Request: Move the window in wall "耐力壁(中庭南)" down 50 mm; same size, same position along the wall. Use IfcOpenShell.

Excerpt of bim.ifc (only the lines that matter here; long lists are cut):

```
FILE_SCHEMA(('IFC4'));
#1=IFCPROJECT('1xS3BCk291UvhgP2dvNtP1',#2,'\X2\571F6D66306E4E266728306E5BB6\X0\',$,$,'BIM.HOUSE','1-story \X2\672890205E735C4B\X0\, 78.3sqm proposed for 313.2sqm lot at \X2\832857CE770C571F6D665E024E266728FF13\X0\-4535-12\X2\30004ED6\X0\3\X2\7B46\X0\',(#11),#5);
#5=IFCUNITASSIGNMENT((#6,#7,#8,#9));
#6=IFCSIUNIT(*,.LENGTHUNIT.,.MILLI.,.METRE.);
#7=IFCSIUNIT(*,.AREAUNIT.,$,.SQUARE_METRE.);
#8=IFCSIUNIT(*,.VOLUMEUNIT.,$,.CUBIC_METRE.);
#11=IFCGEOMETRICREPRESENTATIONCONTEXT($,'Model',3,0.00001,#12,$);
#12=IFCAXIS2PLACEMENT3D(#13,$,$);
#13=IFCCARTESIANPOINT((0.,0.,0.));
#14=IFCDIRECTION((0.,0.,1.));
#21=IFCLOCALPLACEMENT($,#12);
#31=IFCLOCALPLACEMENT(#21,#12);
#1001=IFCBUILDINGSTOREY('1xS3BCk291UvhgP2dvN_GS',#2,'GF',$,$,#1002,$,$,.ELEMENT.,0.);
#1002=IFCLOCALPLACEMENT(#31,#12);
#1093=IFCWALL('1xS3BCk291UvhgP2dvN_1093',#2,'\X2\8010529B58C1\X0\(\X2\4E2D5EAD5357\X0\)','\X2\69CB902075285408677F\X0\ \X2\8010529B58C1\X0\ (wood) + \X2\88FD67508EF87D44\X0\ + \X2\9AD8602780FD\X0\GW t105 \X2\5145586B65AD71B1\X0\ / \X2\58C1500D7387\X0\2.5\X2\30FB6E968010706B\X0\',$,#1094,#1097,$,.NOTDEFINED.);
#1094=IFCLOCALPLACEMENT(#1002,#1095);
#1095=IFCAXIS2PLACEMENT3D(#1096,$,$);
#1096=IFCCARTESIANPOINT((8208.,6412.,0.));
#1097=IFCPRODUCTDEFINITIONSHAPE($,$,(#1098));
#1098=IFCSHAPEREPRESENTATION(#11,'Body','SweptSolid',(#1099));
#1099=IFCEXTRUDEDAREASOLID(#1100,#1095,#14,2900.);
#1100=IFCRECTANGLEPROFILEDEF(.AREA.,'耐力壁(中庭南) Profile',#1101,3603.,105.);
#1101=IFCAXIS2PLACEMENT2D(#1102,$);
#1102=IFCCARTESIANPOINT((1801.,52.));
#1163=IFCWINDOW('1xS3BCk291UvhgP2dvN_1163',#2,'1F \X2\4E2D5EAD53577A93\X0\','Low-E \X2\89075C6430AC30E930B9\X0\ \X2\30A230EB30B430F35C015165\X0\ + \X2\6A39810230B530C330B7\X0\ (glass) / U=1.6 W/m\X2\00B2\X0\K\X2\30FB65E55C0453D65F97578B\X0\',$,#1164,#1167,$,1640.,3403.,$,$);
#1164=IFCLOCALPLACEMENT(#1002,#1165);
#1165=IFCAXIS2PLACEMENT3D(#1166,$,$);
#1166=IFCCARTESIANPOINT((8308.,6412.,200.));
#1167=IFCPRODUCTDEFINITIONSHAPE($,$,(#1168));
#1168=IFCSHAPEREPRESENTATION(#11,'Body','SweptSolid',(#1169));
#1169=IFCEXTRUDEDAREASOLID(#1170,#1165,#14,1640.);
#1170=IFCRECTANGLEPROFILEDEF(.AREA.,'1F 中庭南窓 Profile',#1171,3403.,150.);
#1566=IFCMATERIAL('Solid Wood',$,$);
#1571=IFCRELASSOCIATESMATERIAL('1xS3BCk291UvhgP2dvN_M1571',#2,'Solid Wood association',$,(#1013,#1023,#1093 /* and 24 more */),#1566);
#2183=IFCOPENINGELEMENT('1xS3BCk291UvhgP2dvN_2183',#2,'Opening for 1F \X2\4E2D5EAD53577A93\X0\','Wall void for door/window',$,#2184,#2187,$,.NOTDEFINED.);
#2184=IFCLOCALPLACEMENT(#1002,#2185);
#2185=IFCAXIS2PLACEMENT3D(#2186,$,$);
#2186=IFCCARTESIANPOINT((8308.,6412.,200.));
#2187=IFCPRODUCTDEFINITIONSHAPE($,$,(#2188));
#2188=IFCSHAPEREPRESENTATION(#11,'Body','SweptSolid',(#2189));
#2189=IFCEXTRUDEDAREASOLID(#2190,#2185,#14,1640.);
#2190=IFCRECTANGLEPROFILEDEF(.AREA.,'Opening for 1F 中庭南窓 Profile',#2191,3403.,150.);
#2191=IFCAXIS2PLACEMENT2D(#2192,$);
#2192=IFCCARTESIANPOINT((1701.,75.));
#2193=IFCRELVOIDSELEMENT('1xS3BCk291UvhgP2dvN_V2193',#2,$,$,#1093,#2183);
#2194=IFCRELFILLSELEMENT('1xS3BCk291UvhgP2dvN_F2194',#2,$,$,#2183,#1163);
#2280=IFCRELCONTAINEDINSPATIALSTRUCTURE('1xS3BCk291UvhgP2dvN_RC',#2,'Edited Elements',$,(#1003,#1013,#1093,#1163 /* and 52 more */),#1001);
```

```python
import numpy as np
import ifcopenshell
import ifcopenshell.api.geometry
import ifcopenshell.util.placement
import ifcopenshell.util.unit

model = ifcopenshell.open("bim.ifc")
unit_scale = ifcopenshell.util.unit.calculate_unit_scale(model)

window = model.by_guid("1xS3BCk291UvhgP2dvN_1163")
opening = window.FillsVoids[0].RelatingOpeningElement
dz = -50.0

shift = np.array([0.0, 0.0, dz])
# The window is not placed relative to its opening, so move both.
for product in (opening, window):
    matrix = ifcopenshell.util.placement.get_local_placement(product.ObjectPlacement)
    matrix[:3, 3] += shift
    ifcopenshell.api.geometry.edit_object_placement(model, product=product, matrix=matrix, is_si=False)

print(f"moved by {dz * unit_scale:+.3f} m")

model.write("bim_edited.ifc")
```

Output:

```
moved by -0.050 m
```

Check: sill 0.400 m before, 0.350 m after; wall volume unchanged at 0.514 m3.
